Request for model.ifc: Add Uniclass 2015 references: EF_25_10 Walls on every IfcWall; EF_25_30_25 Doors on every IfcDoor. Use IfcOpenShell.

First a look at what the model holds.

```python
import ifcopenshell

model = ifcopenshell.open("model.ifc")
print(model.schema)
print("classifications:", [c.Name for c in model.by_type("IfcClassification")])
for ifc_class in ("IfcDoor", "IfcRoof", "IfcStair", "IfcWall", "IfcWindow"):
    print(ifc_class, len(model.by_type(ifc_class)))
```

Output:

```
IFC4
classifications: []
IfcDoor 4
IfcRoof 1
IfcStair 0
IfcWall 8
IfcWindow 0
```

```python
import ifcopenshell
import ifcopenshell.api.classification

model = ifcopenshell.open("model.ifc")

system = ifcopenshell.api.classification.add_classification(model, classification="Uniclass 2015")

codes = {
    "IfcWall": ("EF_25_10", "Walls"),
    "IfcDoor": ("EF_25_30_25", "Doors"),
}
for ifc_class, (code, name) in codes.items():
    products = model.by_type(ifc_class)
    ifcopenshell.api.classification.add_reference(
        model, products=products, classification=system, identification=code, name=name
    )
    print(code, len(products))

model.write("model_updated.ifc")
```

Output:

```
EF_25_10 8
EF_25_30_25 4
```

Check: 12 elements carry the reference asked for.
